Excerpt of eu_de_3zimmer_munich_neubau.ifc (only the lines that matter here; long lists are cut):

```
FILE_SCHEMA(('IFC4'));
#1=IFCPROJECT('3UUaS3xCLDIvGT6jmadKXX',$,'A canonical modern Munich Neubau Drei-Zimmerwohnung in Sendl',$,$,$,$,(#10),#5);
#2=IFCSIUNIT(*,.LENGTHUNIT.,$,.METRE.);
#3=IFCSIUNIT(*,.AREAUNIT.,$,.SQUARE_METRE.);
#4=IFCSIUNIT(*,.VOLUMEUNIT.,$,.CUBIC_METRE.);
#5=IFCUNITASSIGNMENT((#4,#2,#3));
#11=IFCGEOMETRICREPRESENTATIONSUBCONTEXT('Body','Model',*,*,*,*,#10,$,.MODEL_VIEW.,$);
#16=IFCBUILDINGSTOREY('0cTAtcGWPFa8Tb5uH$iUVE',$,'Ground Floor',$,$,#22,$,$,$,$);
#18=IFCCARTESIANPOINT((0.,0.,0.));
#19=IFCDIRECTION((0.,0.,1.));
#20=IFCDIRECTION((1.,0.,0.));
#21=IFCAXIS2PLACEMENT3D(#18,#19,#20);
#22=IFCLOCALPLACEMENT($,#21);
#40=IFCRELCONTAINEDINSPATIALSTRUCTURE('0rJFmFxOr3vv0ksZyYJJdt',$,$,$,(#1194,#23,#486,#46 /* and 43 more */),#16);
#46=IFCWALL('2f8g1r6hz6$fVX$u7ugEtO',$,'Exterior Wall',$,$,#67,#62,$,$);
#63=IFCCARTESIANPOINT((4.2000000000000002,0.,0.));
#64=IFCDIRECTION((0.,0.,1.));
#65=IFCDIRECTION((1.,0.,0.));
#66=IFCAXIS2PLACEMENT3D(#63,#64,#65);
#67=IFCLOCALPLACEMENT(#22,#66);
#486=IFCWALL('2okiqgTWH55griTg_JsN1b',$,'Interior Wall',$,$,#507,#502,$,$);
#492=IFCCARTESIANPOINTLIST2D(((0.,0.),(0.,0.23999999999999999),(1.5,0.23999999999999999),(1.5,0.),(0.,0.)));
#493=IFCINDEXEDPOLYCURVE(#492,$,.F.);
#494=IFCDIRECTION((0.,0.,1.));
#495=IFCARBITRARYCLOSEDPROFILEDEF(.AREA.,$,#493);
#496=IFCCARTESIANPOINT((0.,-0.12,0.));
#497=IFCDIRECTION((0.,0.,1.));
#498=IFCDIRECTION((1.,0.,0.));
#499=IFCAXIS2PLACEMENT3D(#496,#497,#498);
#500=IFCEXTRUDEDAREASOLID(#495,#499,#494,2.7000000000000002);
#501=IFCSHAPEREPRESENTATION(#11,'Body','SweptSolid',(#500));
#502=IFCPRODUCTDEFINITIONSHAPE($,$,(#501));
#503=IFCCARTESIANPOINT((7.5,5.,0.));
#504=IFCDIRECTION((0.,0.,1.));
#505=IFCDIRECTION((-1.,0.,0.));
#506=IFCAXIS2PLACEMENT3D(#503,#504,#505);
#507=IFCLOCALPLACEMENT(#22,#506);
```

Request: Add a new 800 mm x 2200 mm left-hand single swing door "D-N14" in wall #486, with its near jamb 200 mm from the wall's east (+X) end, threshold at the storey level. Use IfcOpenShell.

```python
import numpy as np
import ifcopenshell
import ifcopenshell.api.feature
import ifcopenshell.api.geometry
import ifcopenshell.api.root
import ifcopenshell.api.spatial
import ifcopenshell.geom
import ifcopenshell.util.element
import ifcopenshell.util.placement
import ifcopenshell.util.representation
import ifcopenshell.util.shape
import ifcopenshell.util.unit

model = ifcopenshell.open("eu_de_3zimmer_munich_neubau.ifc")
unit_scale = ifcopenshell.util.unit.calculate_unit_scale(model)
settings = ifcopenshell.geom.settings()


def volume(element):
    """Net volume in cubic metres, openings subtracted."""
    shape = ifcopenshell.geom.create_shape(settings, element)
    return ifcopenshell.util.shape.get_volume(shape.geometry)


wall = model.by_guid("2okiqgTWH55griTg_JsN1b")
storey = ifcopenshell.util.element.get_container(wall, ifc_class="IfcBuildingStorey")
context = ifcopenshell.util.representation.get_context(model, "Model", "Body", "MODEL_VIEW")
before = volume(wall)

width, height, from_end, sill = 0.8, 2.2, 0.2, 0.0  # metres

# The wall runs along its own X axis, and the end named is its -X end.
wall_shape = ifcopenshell.geom.create_shape(settings, wall)
x, y, z = ifcopenshell.util.shape.get_vertices(wall_shape.geometry).T
start = x.min() + from_end
face, thickness = float(y.min()), float(y.max() - y.min())
wall_matrix = ifcopenshell.util.placement.get_local_placement(wall.ObjectPlacement)
level = ifcopenshell.util.placement.get_local_placement(storey.ObjectPlacement)[2, 3]


def in_wall(x, y):
    """Placement at x, y metres in the wall's axes, at sill height."""
    matrix = wall_matrix.copy()
    matrix[:, 3] = wall_matrix @ np.array([x / unit_scale, y / unit_scale, 0.0, 1.0])
    matrix[2, 3] = level + sill / unit_scale
    return matrix


# Opening: a box that overshoots both wall faces by 50 mm.
opening = ifcopenshell.api.root.create_entity(model, ifc_class="IfcOpeningElement", predefined_type="OPENING")
box = ifcopenshell.api.geometry.add_wall_representation(
    model, context=context, length=width, height=height, thickness=thickness + 0.1
)
ifcopenshell.api.geometry.assign_representation(model, product=opening, representation=box)
ifcopenshell.api.geometry.edit_object_placement(model, product=opening, matrix=in_wall(start, face - 0.05), is_si=False)
ifcopenshell.api.feature.add_feature(model, feature=opening, element=wall)

door = ifcopenshell.api.root.create_entity(model, ifc_class="IfcDoor", name="D-N14", predefined_type="DOOR")
door.OverallWidth, door.OverallHeight = width / unit_scale, height / unit_scale
door.OperationType = "SINGLE_SWING_LEFT"
body = ifcopenshell.api.geometry.add_door_representation(
    model,
    context=context,
    overall_width=door.OverallWidth,
    overall_height=door.OverallHeight,
    operation_type="SINGLE_SWING_LEFT",
    lining_properties={"LiningDepth": thickness / unit_scale, "ThresholdDepth": thickness / unit_scale},
)
ifcopenshell.api.geometry.assign_representation(model, product=door, representation=body)
ifcopenshell.api.spatial.assign_container(model, products=[door], relating_structure=storey)
ifcopenshell.api.feature.add_filling(model, opening=opening, element=door)

# The lining spans the wall, so the door starts at the wall face.
ifcopenshell.api.geometry.edit_object_placement(model, product=door, matrix=in_wall(start, face), is_si=False)

after = volume(wall)

print(f"wall volume {before:.3f} -> {after:.3f} m3")

model.write("eu_de_3zimmer_munich_neubau_rev.ifc")
```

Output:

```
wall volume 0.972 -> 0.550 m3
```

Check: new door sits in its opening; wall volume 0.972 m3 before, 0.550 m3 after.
